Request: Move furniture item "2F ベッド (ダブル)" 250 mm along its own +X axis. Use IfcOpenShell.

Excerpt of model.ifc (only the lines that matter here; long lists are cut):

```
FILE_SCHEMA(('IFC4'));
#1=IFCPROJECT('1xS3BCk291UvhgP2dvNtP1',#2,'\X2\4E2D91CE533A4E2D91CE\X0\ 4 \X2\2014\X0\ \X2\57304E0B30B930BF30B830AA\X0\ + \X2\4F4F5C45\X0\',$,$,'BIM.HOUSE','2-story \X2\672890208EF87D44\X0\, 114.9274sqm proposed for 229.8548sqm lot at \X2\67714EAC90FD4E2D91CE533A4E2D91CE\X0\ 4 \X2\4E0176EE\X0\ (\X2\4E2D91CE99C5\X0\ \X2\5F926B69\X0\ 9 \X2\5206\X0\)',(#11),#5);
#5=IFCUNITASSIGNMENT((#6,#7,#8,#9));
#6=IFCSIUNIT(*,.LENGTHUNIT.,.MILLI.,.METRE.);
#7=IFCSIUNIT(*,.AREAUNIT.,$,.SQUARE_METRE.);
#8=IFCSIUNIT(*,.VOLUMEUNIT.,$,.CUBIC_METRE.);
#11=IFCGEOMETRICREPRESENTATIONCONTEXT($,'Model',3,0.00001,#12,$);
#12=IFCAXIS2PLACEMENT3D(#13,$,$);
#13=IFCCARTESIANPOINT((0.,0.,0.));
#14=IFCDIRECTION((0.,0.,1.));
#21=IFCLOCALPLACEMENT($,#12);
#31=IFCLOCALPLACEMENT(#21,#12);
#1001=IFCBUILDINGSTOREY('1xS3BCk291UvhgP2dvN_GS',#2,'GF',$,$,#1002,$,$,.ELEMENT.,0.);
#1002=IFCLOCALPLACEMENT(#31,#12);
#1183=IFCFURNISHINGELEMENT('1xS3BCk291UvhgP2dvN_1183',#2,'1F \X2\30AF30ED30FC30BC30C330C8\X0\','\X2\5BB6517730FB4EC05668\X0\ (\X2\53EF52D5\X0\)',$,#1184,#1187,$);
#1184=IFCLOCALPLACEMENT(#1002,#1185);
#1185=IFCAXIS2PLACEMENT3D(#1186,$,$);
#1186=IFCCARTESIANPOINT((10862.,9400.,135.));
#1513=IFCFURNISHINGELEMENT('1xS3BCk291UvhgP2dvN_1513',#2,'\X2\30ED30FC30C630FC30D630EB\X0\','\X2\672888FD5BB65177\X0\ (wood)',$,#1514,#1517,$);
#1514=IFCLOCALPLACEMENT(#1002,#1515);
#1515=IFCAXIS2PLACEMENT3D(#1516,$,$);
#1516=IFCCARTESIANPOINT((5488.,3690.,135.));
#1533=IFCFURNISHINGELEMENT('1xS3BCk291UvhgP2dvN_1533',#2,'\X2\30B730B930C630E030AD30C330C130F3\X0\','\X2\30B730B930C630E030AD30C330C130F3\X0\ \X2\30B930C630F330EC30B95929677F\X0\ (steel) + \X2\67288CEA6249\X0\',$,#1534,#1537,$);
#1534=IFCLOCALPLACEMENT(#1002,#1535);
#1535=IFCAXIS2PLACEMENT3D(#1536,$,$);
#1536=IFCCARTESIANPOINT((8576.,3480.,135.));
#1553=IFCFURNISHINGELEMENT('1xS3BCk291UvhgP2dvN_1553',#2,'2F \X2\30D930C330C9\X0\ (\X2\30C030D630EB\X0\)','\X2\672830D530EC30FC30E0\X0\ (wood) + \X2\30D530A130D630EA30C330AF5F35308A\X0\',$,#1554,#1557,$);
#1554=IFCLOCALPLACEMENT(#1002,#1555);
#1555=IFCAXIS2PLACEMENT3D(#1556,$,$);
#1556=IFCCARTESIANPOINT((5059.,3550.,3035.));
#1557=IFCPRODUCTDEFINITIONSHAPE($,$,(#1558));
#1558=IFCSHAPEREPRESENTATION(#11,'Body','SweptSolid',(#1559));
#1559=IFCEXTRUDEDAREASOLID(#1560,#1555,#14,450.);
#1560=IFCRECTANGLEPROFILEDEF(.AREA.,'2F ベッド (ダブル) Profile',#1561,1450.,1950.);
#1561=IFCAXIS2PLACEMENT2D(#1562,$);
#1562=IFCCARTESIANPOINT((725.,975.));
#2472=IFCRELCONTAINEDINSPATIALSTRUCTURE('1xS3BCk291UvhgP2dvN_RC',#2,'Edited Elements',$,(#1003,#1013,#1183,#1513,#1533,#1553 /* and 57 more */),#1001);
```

```python
import ifcopenshell
import ifcopenshell.api.geometry
import ifcopenshell.util.placement
import ifcopenshell.util.unit

model = ifcopenshell.open("model.ifc")
unit_scale = ifcopenshell.util.unit.calculate_unit_scale(model)

item = model.by_guid("1xS3BCk291UvhgP2dvN_1553")
matrix = ifcopenshell.util.placement.get_local_placement(item.ObjectPlacement)
matrix[:3, 3] += matrix[:3, 0] * 0.25 / unit_scale
ifcopenshell.api.geometry.edit_object_placement(model, product=item, matrix=matrix, is_si=False)

print(ifcopenshell.util.placement.get_local_placement(item.ObjectPlacement).round(3) + 0.0)

model.write("model_updated.ifc")
```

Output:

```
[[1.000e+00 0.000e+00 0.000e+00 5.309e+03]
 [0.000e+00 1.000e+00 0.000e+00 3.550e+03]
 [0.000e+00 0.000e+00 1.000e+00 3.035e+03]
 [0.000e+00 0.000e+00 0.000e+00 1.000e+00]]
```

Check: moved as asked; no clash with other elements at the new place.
